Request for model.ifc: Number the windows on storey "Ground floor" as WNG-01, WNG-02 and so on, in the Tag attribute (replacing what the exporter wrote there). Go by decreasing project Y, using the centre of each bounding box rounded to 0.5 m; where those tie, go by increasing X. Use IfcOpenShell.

First a look at what the model holds.

```python
import ifcopenshell
import ifcopenshell.util.element
import ifcopenshell.util.placement

model = ifcopenshell.open("model.ifc")
print(model.schema)
storey = next(s for s in model.by_type("IfcBuildingStorey") if s.Name == "Ground floor")
windows = [e for e in ifcopenshell.util.element.get_decomposition(storey) if e.is_a("IfcWindow")]
for e in sorted(windows, key=lambda e: e.id()):
    origin = ifcopenshell.util.placement.get_local_placement(e.ObjectPlacement)[:3, 3]
    print(e.id(), e.Tag, e.Name, origin.round(2) + 0.0, sep=" | ")
```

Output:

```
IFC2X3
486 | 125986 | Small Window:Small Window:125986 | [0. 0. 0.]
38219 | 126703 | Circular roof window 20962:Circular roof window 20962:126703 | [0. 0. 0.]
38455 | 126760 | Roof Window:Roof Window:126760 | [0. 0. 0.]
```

```python
import ifcopenshell
import ifcopenshell.geom
import ifcopenshell.util.element
import ifcopenshell.util.shape

model = ifcopenshell.open("model.ifc")
settings = ifcopenshell.geom.settings()
settings.set("use-world-coords", True)


def centre(element):
    shape = ifcopenshell.geom.create_shape(settings, element)
    return ifcopenshell.util.shape.get_bbox_centroid(shape.geometry)


storey = next(s for s in model.by_type("IfcBuildingStorey") if s.Name == "Ground floor")
windows = [e for e in ifcopenshell.util.element.get_decomposition(storey) if e.is_a("IfcWindow")]

# Insertion points can sit at a corner or the storey origin, so sort by the geometry (in metres).
centres = {e: centre(e) for e in windows}
windows.sort(key=lambda e: (-round(centres[e][1] / 0.5), centres[e][0]))

for i, e in enumerate(windows, start=1):
    number = f"WNG-{i:02d}"
    e.Tag = number
    print(e.id(), number)

model.write("model_edited.ifc")
```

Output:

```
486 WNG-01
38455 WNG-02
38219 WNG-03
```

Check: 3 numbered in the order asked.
